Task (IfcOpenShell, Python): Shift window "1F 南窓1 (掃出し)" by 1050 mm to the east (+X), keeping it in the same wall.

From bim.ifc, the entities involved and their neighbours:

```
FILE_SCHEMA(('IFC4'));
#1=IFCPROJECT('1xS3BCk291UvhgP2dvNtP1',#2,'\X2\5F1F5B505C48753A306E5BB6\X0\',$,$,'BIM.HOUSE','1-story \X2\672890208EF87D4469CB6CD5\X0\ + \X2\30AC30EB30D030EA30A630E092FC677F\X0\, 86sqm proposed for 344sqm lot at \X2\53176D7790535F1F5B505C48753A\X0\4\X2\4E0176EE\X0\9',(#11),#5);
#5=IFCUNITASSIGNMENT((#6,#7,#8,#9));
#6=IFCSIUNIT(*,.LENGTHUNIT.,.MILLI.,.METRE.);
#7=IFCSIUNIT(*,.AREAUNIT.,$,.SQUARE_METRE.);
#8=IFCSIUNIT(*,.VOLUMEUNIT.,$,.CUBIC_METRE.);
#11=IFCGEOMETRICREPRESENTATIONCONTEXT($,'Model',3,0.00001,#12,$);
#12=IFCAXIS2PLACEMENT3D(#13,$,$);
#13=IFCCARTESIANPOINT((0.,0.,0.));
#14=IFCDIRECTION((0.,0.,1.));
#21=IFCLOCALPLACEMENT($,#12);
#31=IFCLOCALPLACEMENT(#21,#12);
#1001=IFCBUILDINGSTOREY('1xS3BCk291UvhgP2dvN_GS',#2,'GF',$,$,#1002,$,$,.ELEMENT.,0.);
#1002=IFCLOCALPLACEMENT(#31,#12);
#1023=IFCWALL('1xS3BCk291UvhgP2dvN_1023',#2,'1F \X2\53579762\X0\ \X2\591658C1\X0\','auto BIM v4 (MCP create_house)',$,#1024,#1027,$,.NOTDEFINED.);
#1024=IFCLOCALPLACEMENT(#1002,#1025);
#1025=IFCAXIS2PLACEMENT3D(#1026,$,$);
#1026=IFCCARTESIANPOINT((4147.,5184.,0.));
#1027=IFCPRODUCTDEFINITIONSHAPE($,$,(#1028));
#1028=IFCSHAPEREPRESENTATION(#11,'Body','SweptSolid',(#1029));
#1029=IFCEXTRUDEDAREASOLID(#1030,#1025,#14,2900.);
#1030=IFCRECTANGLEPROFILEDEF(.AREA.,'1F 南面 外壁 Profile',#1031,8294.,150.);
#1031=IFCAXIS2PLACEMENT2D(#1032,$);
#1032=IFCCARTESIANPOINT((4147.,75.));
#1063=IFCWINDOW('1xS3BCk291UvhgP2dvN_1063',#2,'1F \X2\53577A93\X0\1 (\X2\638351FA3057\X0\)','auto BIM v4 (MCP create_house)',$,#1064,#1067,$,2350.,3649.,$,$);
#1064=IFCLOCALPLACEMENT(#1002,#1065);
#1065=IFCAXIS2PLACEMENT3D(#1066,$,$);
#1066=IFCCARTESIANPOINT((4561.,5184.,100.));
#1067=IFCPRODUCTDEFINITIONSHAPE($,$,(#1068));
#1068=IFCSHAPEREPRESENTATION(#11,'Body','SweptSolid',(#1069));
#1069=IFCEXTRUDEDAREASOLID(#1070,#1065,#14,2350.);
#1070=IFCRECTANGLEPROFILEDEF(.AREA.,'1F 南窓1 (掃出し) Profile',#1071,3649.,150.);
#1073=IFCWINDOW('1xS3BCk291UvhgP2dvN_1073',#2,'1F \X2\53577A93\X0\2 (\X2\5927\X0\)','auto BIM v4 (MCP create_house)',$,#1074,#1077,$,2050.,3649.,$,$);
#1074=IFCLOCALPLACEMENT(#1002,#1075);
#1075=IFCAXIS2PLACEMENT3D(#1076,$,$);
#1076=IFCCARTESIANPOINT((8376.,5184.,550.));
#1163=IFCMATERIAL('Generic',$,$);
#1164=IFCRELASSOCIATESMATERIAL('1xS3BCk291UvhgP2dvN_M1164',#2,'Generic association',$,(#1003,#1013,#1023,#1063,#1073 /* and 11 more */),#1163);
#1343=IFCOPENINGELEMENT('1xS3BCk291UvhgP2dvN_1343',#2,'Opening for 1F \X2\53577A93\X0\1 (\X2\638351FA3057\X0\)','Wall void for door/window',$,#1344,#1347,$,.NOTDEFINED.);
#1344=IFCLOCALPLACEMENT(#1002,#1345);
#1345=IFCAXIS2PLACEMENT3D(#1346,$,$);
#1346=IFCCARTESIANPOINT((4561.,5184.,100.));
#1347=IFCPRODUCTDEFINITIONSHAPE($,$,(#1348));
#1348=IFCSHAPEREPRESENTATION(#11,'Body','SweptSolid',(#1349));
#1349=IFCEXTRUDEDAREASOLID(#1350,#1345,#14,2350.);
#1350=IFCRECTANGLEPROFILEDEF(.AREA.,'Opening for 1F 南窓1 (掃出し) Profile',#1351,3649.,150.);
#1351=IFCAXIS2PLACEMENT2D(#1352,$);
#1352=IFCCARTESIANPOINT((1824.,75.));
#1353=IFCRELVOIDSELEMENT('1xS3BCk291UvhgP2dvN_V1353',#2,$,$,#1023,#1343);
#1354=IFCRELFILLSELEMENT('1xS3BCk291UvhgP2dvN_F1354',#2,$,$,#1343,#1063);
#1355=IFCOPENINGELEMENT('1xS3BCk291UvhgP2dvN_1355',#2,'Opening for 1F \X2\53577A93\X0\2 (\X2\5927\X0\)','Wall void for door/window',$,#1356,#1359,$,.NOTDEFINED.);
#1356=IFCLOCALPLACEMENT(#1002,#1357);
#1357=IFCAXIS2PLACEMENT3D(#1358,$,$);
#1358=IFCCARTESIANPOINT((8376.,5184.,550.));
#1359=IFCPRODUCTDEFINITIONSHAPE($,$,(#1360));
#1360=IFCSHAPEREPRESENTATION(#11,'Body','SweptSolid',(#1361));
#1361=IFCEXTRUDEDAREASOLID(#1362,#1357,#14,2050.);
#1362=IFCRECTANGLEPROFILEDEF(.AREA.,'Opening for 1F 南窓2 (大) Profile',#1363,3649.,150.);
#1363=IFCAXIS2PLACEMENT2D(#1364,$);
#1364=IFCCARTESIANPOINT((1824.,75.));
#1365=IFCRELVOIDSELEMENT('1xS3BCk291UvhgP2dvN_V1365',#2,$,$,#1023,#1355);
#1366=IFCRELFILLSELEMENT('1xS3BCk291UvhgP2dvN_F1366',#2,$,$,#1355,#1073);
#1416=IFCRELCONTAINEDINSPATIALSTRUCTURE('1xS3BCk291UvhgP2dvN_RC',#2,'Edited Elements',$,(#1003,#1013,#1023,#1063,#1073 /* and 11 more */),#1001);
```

```python
import ifcopenshell
import ifcopenshell.api.geometry
import ifcopenshell.util.placement
import ifcopenshell.util.unit

model = ifcopenshell.open("bim.ifc")
unit_scale = ifcopenshell.util.unit.calculate_unit_scale(model)

window = model.by_guid("1xS3BCk291UvhgP2dvN_1063")
opening = window.FillsVoids[0].RelatingOpeningElement
wall = opening.VoidsElements[0].RelatingBuildingElement

wall_matrix = ifcopenshell.util.placement.get_local_placement(wall.ObjectPlacement)
shift = wall_matrix[:3, 0] * 1.05 / unit_scale
before = ifcopenshell.util.placement.get_local_placement(window.ObjectPlacement)[:3, 3].copy()

# The window is not placed relative to its opening, so move both.
for product in (opening, window):
    matrix = ifcopenshell.util.placement.get_local_placement(product.ObjectPlacement)
    matrix[:3, 3] += shift
    ifcopenshell.api.geometry.edit_object_placement(model, product=product, matrix=matrix, is_si=False)

after = ifcopenshell.util.placement.get_local_placement(window.ObjectPlacement)[:3, 3]
print("window moved by", (after - before).round(3) + 0.0)

model.write("bim-out.ifc")
```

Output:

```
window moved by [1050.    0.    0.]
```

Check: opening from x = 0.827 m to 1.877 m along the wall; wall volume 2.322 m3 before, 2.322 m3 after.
